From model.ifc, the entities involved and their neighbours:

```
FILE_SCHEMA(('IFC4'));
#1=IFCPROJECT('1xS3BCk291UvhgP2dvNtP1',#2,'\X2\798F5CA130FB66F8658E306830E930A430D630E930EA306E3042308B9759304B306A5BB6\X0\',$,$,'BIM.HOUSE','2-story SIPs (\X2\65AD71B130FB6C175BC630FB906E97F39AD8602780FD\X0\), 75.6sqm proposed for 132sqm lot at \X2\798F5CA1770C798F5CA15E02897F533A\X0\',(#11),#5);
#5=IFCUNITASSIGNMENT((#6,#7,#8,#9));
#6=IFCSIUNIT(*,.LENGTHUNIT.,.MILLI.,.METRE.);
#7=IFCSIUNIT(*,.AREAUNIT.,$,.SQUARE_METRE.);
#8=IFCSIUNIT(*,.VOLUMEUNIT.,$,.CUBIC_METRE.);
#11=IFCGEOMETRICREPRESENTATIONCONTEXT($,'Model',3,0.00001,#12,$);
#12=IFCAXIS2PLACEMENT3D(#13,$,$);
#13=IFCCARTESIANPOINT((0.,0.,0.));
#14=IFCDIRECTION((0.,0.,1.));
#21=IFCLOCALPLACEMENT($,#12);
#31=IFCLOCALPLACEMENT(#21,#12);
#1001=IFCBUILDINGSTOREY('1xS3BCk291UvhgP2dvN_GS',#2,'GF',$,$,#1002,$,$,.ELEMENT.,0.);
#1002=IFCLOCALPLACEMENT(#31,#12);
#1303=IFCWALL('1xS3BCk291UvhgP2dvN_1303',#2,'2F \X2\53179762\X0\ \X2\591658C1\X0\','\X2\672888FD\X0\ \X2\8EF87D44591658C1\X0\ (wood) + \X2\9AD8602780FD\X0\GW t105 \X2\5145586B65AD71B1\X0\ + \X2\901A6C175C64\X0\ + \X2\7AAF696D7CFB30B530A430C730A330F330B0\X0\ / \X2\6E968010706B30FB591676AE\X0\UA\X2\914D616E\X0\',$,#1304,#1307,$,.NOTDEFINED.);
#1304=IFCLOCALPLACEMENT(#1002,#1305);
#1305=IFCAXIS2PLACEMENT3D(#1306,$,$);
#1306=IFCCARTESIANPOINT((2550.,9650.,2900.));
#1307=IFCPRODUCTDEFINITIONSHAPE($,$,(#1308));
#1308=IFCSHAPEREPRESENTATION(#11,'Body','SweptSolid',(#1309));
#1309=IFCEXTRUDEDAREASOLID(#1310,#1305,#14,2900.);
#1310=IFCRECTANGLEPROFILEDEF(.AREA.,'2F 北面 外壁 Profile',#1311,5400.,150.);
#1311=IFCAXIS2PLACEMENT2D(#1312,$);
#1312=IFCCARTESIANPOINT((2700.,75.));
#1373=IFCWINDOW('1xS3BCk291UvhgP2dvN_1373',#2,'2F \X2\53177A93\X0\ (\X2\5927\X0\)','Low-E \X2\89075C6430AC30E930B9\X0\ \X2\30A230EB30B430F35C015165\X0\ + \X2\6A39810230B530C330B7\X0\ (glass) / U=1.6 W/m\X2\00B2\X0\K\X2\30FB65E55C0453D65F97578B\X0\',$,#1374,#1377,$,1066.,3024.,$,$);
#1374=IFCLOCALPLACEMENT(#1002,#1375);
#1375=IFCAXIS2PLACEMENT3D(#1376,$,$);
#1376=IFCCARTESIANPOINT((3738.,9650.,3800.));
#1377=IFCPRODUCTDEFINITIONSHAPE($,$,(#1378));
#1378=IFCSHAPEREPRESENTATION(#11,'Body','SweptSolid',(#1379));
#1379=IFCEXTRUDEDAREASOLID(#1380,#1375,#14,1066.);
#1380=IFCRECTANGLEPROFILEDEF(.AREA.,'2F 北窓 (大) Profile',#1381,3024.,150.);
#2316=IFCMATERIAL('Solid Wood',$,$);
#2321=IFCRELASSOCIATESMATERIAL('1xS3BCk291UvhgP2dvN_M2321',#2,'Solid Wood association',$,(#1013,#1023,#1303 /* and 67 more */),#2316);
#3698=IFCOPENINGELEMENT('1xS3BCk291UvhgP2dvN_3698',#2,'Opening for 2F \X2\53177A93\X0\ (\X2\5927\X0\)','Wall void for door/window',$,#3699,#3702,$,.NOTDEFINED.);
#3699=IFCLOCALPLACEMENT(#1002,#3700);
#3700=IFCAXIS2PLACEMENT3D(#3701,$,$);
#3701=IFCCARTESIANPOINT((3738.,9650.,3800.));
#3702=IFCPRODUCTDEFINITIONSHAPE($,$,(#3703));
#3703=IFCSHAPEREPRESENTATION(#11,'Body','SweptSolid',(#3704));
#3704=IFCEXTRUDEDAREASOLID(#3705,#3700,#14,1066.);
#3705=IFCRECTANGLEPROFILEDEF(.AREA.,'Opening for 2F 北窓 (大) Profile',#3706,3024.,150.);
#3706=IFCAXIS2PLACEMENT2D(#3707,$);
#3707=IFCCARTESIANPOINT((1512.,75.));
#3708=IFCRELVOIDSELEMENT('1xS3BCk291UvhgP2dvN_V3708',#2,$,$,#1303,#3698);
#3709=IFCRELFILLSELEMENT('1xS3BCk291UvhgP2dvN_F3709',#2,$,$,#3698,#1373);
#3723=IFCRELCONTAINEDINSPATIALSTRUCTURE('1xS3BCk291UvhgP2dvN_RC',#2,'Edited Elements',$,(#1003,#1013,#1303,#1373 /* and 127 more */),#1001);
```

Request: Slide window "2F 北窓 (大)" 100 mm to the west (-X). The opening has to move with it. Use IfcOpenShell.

```python
import ifcopenshell
import ifcopenshell.api.geometry
import ifcopenshell.util.placement

model = ifcopenshell.open("model.ifc")

window = model.by_id(1373)
opening = window.FillsVoids[0].RelatingOpeningElement
wall = opening.VoidsElements[0].RelatingBuildingElement

wall_matrix = ifcopenshell.util.placement.get_local_placement(wall.ObjectPlacement)
shift = wall_matrix[:3, 0] * -100.0
before = ifcopenshell.util.placement.get_local_placement(window.ObjectPlacement)[:3, 3].copy()

# The window is not placed relative to its opening, so move both.
for product in (opening, window):
    matrix = ifcopenshell.util.placement.get_local_placement(product.ObjectPlacement)
    matrix[:3, 3] += shift
    ifcopenshell.api.geometry.edit_object_placement(model, product=product, matrix=matrix, is_si=False)

after = ifcopenshell.util.placement.get_local_placement(window.ObjectPlacement)[:3, 3]
print("window moved by", (after - before).round(3) + 0.0)

model.write("model_edited.ifc")
```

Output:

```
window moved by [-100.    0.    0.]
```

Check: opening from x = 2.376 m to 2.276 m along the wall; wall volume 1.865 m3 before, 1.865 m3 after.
